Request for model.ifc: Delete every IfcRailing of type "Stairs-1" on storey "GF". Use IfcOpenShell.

First a look at what the model holds.

```python
import ifcopenshell
import ifcopenshell.util.element

model = ifcopenshell.open("model.ifc")
print(model.schema)
storey = next(s for s in model.by_type("IfcBuildingStorey") if s.Name == "GF")
railings = [e for e in ifcopenshell.util.element.get_decomposition(storey) if e.is_a("IfcRailing")]
seen = {}
for e in railings:
    element_type = ifcopenshell.util.element.get_type(e)
    name = element_type.Name if element_type not in (None, e) else None
    seen[name] = seen.get(name, 0) + 1
for name, count in sorted(seen.items(), key=str):
    print(count, "x", name)
```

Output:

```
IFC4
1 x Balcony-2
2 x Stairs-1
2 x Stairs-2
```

```python
import ifcopenshell
import ifcopenshell.api.root
import ifcopenshell.util.element

model = ifcopenshell.open("model.ifc")

storey = next(s for s in model.by_type("IfcBuildingStorey") if s.Name == "GF")
railings = [e for e in ifcopenshell.util.element.get_decomposition(storey) if e.is_a("IfcRailing")]
targets = [e for e in railings if (t := ifcopenshell.util.element.get_type(e)) not in (None, e) and t.Name == "Stairs-1"]

for e in targets:
    ifcopenshell.api.root.remove_product(model, product=e)
print(len(targets), "removed")

model.write("model_edited.ifc")
```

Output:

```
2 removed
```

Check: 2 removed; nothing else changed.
